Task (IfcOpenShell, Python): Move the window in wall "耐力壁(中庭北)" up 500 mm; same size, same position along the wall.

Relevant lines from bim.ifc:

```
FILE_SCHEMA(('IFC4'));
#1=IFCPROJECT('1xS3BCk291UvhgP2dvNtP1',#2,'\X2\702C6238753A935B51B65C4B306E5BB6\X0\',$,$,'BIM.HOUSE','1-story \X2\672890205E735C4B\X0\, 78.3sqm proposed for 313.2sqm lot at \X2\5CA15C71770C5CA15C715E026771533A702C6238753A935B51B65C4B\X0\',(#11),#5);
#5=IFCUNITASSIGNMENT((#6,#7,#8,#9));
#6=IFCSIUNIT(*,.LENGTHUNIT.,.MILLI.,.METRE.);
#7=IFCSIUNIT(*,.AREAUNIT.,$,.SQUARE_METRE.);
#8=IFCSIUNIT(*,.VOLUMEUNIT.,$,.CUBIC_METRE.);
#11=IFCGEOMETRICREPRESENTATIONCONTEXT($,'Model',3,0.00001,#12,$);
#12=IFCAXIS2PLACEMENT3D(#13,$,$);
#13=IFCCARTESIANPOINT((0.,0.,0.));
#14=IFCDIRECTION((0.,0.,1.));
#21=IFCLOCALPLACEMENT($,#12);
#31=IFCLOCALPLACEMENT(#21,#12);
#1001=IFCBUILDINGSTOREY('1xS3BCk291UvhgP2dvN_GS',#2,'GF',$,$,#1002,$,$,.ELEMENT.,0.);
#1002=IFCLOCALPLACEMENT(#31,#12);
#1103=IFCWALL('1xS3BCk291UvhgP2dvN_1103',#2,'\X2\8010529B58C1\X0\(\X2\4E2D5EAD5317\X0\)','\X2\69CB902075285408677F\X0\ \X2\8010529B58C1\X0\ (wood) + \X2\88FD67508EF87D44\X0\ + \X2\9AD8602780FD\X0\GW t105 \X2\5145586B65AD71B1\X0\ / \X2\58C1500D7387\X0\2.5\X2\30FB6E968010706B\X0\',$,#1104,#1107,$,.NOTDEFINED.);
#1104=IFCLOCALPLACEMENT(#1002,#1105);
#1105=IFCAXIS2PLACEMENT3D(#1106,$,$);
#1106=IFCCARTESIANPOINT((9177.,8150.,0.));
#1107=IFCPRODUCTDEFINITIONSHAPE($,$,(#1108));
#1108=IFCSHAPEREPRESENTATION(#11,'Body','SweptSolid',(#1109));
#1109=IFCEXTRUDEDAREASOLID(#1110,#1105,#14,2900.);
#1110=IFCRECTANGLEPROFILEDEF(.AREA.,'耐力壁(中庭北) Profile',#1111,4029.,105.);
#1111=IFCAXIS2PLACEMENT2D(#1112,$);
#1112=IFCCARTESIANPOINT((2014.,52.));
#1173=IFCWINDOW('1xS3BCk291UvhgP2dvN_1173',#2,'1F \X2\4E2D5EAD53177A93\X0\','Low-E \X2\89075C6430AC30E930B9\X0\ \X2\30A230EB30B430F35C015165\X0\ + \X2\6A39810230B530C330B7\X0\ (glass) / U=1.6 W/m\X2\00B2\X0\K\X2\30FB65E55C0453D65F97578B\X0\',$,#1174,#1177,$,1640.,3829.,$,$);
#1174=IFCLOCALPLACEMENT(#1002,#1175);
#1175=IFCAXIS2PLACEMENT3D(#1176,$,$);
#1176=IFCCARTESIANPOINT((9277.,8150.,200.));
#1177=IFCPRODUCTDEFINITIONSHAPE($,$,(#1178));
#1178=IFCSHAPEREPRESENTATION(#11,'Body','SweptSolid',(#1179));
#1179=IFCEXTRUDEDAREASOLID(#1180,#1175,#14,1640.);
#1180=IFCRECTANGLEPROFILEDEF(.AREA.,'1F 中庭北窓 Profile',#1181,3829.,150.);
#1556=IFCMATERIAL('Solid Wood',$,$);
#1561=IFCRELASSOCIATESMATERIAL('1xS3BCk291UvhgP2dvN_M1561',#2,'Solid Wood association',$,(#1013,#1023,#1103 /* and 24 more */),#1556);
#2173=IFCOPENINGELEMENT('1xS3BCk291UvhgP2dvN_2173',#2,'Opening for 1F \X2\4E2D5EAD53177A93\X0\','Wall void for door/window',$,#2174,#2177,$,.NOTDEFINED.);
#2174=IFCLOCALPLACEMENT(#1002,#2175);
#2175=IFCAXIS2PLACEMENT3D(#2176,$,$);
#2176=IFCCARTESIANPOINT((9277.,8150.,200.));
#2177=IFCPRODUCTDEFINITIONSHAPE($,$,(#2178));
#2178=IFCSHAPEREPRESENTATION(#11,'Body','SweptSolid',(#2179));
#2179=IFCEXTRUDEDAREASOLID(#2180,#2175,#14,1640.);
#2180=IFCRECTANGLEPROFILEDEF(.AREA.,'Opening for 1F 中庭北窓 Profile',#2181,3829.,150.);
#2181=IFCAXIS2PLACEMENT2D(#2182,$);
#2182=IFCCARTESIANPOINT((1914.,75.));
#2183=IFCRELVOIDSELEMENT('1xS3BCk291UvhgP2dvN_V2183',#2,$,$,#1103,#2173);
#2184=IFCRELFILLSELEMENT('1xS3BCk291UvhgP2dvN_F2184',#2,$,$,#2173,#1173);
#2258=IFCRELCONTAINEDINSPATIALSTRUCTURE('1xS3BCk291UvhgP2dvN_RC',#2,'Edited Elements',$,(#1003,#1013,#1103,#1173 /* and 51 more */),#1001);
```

```python
import numpy as np
import ifcopenshell
import ifcopenshell.api.geometry
import ifcopenshell.util.placement
import ifcopenshell.util.unit

model = ifcopenshell.open("bim.ifc")
unit_scale = ifcopenshell.util.unit.calculate_unit_scale(model)

window = model.by_id(1173)
opening = window.FillsVoids[0].RelatingOpeningElement
dz = 0.5 / unit_scale

shift = np.array([0.0, 0.0, dz])
# The window is not placed relative to its opening, so move both.
for product in (opening, window):
    matrix = ifcopenshell.util.placement.get_local_placement(product.ObjectPlacement)
    matrix[:3, 3] += shift
    ifcopenshell.api.geometry.edit_object_placement(model, product=product, matrix=matrix, is_si=False)

print(f"moved by {dz * unit_scale:+.3f} m")

model.write("bim_updated.ifc")
```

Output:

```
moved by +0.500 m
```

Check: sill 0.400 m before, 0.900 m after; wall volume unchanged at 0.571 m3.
